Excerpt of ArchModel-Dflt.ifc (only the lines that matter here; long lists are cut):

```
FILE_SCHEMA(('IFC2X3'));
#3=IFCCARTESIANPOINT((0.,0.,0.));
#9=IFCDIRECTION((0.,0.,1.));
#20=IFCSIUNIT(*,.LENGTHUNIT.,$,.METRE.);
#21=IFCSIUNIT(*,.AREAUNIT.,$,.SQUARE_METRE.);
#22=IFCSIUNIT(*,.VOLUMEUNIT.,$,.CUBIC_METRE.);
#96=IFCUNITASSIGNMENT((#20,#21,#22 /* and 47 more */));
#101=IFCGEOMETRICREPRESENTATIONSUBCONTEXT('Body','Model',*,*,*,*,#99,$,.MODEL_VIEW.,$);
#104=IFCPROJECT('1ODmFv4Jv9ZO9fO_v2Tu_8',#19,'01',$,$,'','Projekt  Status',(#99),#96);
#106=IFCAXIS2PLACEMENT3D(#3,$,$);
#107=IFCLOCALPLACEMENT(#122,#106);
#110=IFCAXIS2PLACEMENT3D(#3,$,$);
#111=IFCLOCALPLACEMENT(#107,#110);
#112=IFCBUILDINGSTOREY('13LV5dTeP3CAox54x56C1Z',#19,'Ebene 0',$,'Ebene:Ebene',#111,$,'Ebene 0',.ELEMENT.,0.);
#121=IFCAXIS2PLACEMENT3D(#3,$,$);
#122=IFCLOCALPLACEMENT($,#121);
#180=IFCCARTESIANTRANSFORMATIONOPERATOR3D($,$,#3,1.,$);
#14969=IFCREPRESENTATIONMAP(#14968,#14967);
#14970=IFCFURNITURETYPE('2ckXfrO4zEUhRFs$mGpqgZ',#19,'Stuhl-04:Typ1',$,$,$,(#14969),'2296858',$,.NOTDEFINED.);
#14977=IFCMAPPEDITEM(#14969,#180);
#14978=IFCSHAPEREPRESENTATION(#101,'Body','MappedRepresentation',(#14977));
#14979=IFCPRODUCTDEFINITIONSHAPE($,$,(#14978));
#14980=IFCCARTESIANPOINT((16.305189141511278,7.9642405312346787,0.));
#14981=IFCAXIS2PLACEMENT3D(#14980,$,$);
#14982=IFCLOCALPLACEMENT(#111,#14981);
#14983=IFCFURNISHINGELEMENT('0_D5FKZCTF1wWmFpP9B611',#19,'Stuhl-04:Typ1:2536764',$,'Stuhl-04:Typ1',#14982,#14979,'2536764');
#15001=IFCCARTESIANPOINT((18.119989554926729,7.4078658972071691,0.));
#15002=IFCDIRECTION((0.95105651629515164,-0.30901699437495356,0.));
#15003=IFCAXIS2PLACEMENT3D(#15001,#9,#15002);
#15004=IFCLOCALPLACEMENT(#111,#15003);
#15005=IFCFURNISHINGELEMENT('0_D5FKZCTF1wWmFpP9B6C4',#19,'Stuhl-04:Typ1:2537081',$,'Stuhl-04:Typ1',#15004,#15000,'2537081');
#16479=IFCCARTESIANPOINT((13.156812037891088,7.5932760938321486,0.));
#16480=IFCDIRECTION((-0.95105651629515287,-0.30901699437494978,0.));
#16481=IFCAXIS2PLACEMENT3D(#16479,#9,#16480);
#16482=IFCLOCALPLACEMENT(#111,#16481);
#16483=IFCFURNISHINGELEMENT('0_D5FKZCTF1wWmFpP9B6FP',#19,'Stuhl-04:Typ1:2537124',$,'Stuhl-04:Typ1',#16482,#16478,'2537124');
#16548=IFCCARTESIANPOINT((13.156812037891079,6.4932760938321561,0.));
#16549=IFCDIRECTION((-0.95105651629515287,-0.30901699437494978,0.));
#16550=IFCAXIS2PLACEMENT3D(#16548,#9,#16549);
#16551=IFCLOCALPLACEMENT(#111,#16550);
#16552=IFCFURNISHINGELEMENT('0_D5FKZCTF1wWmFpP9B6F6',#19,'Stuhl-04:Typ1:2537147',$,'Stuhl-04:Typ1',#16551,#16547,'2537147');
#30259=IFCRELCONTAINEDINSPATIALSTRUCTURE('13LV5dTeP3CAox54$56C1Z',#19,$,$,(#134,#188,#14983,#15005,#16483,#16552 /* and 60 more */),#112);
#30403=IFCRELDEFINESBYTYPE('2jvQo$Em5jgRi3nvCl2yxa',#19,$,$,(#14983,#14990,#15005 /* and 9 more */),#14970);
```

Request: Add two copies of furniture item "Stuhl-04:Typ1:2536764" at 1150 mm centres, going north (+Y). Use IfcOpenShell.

```python
import numpy as np
import ifcopenshell
import ifcopenshell.api.geometry
import ifcopenshell.api.root
import ifcopenshell.util.element
import ifcopenshell.util.placement
import ifcopenshell.util.unit

model = ifcopenshell.open("ArchModel-Dflt.ifc")
unit_scale = ifcopenshell.util.unit.calculate_unit_scale(model)

source = model.by_guid("0_D5FKZCTF1wWmFpP9B611")
base = ifcopenshell.util.placement.get_local_placement(source.ObjectPlacement)
step = np.array([0.0, 1.0, 0.0]) * 1.15 / unit_scale

for i in range(1, 3):
    copy = ifcopenshell.api.root.copy_class(model, product=source)
    copy.Representation = ifcopenshell.util.element.copy_deep(
        model, source.Representation, exclude=["IfcGeometricRepresentationContext", "IfcRepresentationMap"]
    )
    copy.Name = "Stuhl-04:Typ1"
    copy.Tag = None
    matrix = base.copy()
    matrix[:3, 3] += i * step
    print("added at", matrix[:3, 3].round(3) + 0.0)
    ifcopenshell.api.geometry.edit_object_placement(model, product=copy, matrix=matrix, is_si=False)

model.write("ArchModel-Dflt_v2.ifc")
```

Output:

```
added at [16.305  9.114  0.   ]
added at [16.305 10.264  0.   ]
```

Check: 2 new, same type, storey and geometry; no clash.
